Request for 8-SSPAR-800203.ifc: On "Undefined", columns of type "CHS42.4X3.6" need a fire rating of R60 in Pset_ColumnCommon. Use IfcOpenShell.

First a look at what the model holds.

```python
import ifcopenshell
import ifcopenshell.util.element

model = ifcopenshell.open("8-SSPAR-800203.ifc")
print(model.schema)
storey = next(s for s in model.by_type("IfcBuildingStorey") if s.Name == "Undefined")
columns = [e for e in ifcopenshell.util.element.get_decomposition(storey) if e.is_a("IfcColumn")]
seen = {}
for e in columns:
    element_type = ifcopenshell.util.element.get_type(e)
    key = (element_type.Name if element_type != e and element_type else None, ifcopenshell.util.element.get_pset(e, "Pset_ColumnCommon", "FireRating"))
    seen[key] = seen.get(key, 0) + 1
for (name, value), count in sorted(seen.items(), key=str):
    print(count, "x", name, "|", value)
```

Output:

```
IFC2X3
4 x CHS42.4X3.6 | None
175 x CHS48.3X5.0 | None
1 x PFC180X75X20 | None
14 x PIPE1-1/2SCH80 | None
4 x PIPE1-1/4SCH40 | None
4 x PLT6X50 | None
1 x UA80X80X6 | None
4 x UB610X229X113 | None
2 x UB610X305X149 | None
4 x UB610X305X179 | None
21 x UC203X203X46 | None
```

```python
import ifcopenshell
import ifcopenshell.api.pset
import ifcopenshell.util.element

model = ifcopenshell.open("8-SSPAR-800203.ifc")

storey = next(s for s in model.by_type("IfcBuildingStorey") if s.Name == "Undefined")
columns = [e for e in ifcopenshell.util.element.get_decomposition(storey) if e.is_a("IfcColumn")]

count = 0
for e in columns:
    element_type = ifcopenshell.util.element.get_type(e)
    if element_type in (None, e) or element_type.Name != "CHS42.4X3.6":
        continue
    # add_pset returns the element's existing set when there is one.
    pset = ifcopenshell.api.pset.add_pset(model, product=e, name="Pset_ColumnCommon")
    ifcopenshell.api.pset.edit_pset(model, pset=pset, properties={"FireRating": "R60"})
    count += 1

print(count, "columns updated")

model.write("8-SSPAR-800203_rev.ifc")
```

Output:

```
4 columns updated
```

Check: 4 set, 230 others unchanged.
